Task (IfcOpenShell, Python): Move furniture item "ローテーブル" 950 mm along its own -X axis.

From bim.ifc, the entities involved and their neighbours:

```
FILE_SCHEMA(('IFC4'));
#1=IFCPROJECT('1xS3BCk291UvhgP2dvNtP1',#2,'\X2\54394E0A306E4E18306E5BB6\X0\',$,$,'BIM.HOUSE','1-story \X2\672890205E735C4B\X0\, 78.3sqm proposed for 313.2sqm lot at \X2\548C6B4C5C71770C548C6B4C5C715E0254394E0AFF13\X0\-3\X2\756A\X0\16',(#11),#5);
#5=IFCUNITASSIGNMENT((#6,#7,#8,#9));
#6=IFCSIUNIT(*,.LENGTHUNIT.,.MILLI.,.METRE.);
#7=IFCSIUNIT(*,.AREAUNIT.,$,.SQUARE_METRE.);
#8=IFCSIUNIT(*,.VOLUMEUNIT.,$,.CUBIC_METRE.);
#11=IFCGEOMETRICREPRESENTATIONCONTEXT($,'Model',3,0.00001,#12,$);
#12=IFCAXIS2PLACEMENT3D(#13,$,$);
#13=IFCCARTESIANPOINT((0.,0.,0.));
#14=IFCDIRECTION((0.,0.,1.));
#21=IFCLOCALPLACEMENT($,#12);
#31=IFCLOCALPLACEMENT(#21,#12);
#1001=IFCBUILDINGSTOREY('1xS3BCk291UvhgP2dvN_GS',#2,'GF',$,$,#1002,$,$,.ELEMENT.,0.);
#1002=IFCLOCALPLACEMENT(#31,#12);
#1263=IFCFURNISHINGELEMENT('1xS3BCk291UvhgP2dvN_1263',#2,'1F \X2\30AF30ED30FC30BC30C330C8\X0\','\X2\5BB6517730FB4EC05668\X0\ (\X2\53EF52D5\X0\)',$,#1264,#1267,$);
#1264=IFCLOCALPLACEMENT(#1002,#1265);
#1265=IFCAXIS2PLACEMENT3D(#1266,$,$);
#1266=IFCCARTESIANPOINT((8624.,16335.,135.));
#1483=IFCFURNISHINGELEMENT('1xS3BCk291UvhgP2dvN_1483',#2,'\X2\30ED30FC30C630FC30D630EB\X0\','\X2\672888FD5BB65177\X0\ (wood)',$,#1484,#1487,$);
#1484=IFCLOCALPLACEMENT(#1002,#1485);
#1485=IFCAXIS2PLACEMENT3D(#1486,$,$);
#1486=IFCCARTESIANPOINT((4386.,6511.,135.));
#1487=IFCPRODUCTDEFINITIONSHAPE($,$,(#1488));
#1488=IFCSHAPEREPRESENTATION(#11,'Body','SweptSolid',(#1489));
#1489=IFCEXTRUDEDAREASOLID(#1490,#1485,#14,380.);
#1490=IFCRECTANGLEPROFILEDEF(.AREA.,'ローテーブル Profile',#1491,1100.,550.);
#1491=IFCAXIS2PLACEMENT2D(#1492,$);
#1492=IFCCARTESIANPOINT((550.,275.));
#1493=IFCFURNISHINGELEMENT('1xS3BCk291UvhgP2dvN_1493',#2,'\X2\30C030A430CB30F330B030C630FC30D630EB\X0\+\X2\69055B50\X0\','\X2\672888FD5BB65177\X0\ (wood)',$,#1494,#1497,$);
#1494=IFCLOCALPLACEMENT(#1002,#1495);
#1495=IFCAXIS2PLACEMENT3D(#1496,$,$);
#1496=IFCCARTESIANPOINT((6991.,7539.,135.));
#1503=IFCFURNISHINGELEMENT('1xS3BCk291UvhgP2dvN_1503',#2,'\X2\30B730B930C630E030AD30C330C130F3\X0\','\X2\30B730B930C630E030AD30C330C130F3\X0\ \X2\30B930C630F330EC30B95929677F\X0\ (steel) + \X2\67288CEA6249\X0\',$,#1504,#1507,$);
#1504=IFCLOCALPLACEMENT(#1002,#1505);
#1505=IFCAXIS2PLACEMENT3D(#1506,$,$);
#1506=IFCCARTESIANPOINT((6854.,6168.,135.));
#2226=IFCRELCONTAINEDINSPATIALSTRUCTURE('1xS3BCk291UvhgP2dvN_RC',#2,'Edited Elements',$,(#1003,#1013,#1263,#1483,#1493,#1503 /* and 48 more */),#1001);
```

```python
import ifcopenshell
import ifcopenshell.api.geometry
import ifcopenshell.util.placement
import ifcopenshell.util.unit

model = ifcopenshell.open("bim.ifc")
unit_scale = ifcopenshell.util.unit.calculate_unit_scale(model)

item = model.by_id(1483)
matrix = ifcopenshell.util.placement.get_local_placement(item.ObjectPlacement)
matrix[:3, 3] -= matrix[:3, 0] * 0.95 / unit_scale
ifcopenshell.api.geometry.edit_object_placement(model, product=item, matrix=matrix, is_si=False)

print(ifcopenshell.util.placement.get_local_placement(item.ObjectPlacement).round(3) + 0.0)

model.write("bim_edited.ifc")
```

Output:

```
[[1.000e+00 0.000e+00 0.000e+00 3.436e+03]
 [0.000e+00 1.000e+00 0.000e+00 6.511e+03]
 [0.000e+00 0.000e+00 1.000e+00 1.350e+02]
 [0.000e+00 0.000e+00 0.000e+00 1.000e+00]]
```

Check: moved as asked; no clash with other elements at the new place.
